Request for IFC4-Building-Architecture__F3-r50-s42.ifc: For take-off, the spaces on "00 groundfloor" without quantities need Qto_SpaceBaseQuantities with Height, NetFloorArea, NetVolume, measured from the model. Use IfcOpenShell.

First a look at what the model holds.

```python
import ifcopenshell
import ifcopenshell.util.element
import ifcopenshell.util.unit

model = ifcopenshell.open("IFC4-Building-Architecture__F3-r50-s42.ifc")
print(model.schema)
for unit_type in ("LENGTHUNIT", "AREAUNIT", "VOLUMEUNIT"):
    print(unit_type, ifcopenshell.util.unit.calculate_unit_scale(model, unit_type))
storey = next(s for s in model.by_type("IfcBuildingStorey") if s.Name == "00 groundfloor")
spaces = [e for e in ifcopenshell.util.element.get_decomposition(storey) if e.is_a("IfcSpace")]
for e in sorted(spaces, key=lambda e: e.id()):
    print(e.id(), e.is_a(), e.Name, list(ifcopenshell.util.element.get_psets(e, qtos_only=True)), sep=" | ")
```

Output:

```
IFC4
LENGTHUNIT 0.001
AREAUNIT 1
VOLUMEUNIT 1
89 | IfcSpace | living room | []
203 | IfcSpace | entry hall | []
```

```python
import ifcopenshell
import ifcopenshell.api.pset
import ifcopenshell.geom
import ifcopenshell.util.element
import ifcopenshell.util.shape
import ifcopenshell.util.unit

model = ifcopenshell.open("IFC4-Building-Architecture__F3-r50-s42.ifc")
unit_scale = ifcopenshell.util.unit.calculate_unit_scale(model)
area_scale = ifcopenshell.util.unit.calculate_unit_scale(model, "AREAUNIT")
volume_scale = ifcopenshell.util.unit.calculate_unit_scale(model, "VOLUMEUNIT")
settings = ifcopenshell.geom.settings()

storey = next(s for s in model.by_type("IfcBuildingStorey") if s.Name == "00 groundfloor")
spaces = [e for e in ifcopenshell.util.element.get_decomposition(storey) if e.is_a("IfcSpace")]

for e in sorted(spaces, key=lambda e: e.id()):
    if ifcopenshell.util.element.get_psets(e, qtos_only=True, should_inherit=False):
        continue
    # Geometry comes back in metres, in the element's own axes.
    shape = ifcopenshell.geom.create_shape(settings, e)
    values = {
        "Height": ifcopenshell.util.shape.get_z(shape.geometry) / unit_scale,
        "NetFloorArea": ifcopenshell.util.shape.get_footprint_area(shape.geometry) / area_scale,
        "NetVolume": ifcopenshell.util.shape.get_volume(shape.geometry) / volume_scale,
    }
    qto = ifcopenshell.api.pset.add_qto(model, product=e, name="Qto_SpaceBaseQuantities")
    ifcopenshell.api.pset.edit_qto(model, qto=qto, properties=values)
    print(e.id(), {k: round(v, 3) for k, v in values.items()})

model.write("IFC4-Building-Architecture__F3-r50-s42_rev.ifc")
```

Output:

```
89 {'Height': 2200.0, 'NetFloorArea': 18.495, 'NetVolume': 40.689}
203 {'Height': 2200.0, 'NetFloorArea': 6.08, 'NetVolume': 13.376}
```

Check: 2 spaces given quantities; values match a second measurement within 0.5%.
